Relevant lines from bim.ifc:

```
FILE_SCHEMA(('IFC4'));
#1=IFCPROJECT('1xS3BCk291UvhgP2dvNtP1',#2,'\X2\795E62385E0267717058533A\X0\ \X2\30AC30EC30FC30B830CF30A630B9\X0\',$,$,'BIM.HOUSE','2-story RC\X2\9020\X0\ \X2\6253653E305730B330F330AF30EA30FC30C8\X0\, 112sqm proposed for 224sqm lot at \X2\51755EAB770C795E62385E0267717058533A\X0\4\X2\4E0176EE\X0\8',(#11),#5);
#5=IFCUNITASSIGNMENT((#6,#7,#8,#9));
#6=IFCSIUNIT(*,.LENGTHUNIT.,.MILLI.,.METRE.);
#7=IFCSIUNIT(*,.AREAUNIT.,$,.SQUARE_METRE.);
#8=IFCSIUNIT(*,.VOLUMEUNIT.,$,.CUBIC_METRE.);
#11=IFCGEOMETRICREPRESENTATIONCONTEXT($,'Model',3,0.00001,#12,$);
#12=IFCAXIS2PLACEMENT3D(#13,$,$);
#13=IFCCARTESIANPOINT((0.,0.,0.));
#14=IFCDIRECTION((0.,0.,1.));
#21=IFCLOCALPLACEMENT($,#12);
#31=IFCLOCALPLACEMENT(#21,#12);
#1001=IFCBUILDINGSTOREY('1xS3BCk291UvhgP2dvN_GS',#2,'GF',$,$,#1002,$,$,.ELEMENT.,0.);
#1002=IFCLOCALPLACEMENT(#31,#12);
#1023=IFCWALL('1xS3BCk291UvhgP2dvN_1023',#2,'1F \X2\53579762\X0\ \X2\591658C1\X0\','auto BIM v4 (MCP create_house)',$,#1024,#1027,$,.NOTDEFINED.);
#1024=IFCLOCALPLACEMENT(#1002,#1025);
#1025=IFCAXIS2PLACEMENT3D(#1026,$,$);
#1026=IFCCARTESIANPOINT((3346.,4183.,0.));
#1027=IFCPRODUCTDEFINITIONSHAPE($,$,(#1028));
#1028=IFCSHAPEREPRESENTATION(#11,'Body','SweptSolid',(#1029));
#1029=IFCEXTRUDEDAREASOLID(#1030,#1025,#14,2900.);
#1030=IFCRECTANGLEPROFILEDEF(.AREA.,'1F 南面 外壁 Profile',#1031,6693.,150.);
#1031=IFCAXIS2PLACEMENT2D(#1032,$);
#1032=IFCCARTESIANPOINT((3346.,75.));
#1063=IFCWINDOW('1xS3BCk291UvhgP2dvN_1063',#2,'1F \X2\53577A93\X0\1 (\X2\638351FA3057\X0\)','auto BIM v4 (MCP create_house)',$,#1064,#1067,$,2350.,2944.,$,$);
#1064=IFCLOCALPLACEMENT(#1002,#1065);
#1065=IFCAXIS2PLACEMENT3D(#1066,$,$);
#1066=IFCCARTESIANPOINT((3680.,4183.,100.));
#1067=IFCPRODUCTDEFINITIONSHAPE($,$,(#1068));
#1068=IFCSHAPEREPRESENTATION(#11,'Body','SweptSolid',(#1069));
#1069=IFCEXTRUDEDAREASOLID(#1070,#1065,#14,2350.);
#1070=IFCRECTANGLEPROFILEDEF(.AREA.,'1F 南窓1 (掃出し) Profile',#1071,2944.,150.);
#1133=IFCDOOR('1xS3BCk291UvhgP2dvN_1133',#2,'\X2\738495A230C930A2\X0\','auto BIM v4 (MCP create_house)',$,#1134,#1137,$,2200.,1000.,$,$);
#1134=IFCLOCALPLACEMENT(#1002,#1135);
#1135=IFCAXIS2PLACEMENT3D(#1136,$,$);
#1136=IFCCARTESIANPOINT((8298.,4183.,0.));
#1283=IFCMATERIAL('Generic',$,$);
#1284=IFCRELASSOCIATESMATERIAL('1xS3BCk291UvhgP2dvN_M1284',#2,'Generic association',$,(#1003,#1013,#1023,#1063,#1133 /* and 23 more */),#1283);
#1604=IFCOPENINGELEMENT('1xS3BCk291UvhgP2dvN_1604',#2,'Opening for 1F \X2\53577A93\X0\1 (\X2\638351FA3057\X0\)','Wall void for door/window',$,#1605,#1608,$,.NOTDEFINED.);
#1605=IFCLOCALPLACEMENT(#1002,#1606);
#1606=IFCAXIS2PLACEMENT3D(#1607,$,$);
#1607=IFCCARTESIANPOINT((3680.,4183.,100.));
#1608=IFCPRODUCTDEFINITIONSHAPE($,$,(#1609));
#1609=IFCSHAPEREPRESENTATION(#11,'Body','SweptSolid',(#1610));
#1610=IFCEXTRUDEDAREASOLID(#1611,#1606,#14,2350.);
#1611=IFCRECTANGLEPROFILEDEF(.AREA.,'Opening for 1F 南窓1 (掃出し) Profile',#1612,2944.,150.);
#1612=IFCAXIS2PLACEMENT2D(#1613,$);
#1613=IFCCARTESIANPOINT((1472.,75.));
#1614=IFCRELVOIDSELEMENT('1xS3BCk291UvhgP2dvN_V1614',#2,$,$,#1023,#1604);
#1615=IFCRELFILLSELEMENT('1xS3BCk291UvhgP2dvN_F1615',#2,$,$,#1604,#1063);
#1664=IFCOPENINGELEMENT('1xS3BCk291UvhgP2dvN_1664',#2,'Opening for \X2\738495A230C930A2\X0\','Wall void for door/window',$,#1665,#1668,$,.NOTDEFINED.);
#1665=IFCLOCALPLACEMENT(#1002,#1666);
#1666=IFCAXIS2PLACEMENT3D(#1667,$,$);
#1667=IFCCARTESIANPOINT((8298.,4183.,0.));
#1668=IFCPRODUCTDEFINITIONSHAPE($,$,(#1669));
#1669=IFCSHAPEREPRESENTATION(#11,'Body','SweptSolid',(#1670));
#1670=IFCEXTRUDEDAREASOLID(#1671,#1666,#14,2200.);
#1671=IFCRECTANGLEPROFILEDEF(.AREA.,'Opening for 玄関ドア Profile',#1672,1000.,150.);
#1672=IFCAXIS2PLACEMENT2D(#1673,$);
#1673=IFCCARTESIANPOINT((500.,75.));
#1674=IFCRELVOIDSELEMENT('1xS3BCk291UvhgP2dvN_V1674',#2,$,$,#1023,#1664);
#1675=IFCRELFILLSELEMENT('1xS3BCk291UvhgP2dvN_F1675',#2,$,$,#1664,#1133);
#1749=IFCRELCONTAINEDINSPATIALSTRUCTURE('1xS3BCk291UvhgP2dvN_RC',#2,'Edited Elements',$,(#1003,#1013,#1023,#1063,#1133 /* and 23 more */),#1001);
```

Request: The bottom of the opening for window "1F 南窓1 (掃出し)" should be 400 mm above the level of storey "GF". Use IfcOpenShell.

```python
import numpy as np
import ifcopenshell
import ifcopenshell.api.geometry
import ifcopenshell.geom
import ifcopenshell.util.element
import ifcopenshell.util.placement
import ifcopenshell.util.shape
import ifcopenshell.util.unit

model = ifcopenshell.open("bim.ifc")
unit_scale = ifcopenshell.util.unit.calculate_unit_scale(model)

window = model.by_guid("1xS3BCk291UvhgP2dvN_1063")
opening = window.FillsVoids[0].RelatingOpeningElement
storey = ifcopenshell.util.element.get_container(window, ifc_class="IfcBuildingStorey")
level = ifcopenshell.util.placement.get_local_placement(storey.ObjectPlacement)[2, 3]

# The opening's origin need not be at the sill, so measure its lowest point.
shape = ifcopenshell.geom.create_shape(ifcopenshell.geom.settings(), opening)
bottom = ifcopenshell.util.shape.get_shape_bottom_elevation(shape, shape.geometry) / unit_scale
dz = level + 0.4 / unit_scale - bottom

shift = np.array([0.0, 0.0, dz])
# The window is not placed relative to its opening, so move both.
for product in (opening, window):
    matrix = ifcopenshell.util.placement.get_local_placement(product.ObjectPlacement)
    matrix[:3, 3] += shift
    ifcopenshell.api.geometry.edit_object_placement(model, product=product, matrix=matrix, is_si=False)

print(f"moved by {dz * unit_scale:+.3f} m")

model.write("bim_edited.ifc")
```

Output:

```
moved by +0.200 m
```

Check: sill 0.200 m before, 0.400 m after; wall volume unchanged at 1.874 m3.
